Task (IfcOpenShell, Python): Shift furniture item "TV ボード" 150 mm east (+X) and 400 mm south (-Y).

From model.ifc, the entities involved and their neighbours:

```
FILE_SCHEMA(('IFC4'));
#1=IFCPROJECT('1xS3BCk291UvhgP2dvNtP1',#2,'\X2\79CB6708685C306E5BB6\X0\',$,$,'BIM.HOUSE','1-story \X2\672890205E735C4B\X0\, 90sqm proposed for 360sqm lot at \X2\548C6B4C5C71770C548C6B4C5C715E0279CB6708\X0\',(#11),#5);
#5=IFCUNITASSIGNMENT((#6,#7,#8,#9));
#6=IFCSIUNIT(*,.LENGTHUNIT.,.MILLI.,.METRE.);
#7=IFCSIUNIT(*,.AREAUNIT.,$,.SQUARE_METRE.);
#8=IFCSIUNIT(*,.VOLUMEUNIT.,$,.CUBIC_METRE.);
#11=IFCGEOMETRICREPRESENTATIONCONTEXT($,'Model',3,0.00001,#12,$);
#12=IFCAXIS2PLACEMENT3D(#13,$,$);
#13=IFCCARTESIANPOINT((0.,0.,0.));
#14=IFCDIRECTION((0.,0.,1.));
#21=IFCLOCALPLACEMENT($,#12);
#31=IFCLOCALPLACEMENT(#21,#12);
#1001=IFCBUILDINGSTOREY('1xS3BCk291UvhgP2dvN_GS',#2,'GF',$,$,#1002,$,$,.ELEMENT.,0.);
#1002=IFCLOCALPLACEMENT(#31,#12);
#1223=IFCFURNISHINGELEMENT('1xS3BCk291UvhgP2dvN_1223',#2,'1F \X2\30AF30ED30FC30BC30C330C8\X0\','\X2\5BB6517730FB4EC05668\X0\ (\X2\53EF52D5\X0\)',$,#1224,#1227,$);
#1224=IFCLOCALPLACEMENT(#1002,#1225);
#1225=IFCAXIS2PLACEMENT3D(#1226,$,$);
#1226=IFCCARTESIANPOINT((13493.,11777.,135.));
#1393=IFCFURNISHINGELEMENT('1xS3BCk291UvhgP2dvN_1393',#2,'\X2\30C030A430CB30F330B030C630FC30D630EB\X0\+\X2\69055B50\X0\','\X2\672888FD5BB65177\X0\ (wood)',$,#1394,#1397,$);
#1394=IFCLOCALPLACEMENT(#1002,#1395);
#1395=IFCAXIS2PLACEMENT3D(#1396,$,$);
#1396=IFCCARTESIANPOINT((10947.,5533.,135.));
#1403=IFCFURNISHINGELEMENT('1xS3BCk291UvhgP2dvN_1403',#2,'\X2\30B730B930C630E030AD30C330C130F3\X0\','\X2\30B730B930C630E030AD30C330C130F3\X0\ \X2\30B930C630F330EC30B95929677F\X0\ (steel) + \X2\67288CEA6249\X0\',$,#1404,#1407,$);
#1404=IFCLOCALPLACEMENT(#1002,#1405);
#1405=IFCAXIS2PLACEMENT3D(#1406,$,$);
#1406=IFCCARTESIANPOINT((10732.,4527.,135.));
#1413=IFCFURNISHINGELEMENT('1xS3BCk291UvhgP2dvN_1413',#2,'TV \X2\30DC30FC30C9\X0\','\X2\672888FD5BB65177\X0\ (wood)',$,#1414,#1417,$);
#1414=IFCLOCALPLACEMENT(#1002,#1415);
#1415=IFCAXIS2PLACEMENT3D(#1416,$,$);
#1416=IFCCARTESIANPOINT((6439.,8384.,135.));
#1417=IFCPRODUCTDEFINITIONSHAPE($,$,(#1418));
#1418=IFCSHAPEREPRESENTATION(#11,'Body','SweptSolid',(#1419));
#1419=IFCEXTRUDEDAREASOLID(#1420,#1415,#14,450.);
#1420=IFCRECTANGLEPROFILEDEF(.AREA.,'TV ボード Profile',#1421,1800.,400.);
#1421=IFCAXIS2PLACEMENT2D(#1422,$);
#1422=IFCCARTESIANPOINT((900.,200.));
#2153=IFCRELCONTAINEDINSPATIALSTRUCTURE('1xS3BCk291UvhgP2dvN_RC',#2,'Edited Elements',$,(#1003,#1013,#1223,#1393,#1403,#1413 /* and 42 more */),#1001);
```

```python
import ifcopenshell
import ifcopenshell.api.geometry
import ifcopenshell.util.placement
import ifcopenshell.util.unit

model = ifcopenshell.open("model.ifc")
unit_scale = ifcopenshell.util.unit.calculate_unit_scale(model)

item = model.by_guid("1xS3BCk291UvhgP2dvN_1413")
matrix = ifcopenshell.util.placement.get_local_placement(item.ObjectPlacement)
matrix[0, 3] += 0.15 / unit_scale
matrix[1, 3] -= 0.4 / unit_scale
ifcopenshell.api.geometry.edit_object_placement(model, product=item, matrix=matrix, is_si=False)

print(ifcopenshell.util.placement.get_local_placement(item.ObjectPlacement).round(3) + 0.0)

model.write("model_rev.ifc")
```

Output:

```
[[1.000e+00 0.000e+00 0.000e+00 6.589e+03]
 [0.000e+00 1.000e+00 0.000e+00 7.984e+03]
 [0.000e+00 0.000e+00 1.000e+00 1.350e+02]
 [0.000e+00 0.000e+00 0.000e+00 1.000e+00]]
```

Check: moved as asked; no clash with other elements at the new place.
